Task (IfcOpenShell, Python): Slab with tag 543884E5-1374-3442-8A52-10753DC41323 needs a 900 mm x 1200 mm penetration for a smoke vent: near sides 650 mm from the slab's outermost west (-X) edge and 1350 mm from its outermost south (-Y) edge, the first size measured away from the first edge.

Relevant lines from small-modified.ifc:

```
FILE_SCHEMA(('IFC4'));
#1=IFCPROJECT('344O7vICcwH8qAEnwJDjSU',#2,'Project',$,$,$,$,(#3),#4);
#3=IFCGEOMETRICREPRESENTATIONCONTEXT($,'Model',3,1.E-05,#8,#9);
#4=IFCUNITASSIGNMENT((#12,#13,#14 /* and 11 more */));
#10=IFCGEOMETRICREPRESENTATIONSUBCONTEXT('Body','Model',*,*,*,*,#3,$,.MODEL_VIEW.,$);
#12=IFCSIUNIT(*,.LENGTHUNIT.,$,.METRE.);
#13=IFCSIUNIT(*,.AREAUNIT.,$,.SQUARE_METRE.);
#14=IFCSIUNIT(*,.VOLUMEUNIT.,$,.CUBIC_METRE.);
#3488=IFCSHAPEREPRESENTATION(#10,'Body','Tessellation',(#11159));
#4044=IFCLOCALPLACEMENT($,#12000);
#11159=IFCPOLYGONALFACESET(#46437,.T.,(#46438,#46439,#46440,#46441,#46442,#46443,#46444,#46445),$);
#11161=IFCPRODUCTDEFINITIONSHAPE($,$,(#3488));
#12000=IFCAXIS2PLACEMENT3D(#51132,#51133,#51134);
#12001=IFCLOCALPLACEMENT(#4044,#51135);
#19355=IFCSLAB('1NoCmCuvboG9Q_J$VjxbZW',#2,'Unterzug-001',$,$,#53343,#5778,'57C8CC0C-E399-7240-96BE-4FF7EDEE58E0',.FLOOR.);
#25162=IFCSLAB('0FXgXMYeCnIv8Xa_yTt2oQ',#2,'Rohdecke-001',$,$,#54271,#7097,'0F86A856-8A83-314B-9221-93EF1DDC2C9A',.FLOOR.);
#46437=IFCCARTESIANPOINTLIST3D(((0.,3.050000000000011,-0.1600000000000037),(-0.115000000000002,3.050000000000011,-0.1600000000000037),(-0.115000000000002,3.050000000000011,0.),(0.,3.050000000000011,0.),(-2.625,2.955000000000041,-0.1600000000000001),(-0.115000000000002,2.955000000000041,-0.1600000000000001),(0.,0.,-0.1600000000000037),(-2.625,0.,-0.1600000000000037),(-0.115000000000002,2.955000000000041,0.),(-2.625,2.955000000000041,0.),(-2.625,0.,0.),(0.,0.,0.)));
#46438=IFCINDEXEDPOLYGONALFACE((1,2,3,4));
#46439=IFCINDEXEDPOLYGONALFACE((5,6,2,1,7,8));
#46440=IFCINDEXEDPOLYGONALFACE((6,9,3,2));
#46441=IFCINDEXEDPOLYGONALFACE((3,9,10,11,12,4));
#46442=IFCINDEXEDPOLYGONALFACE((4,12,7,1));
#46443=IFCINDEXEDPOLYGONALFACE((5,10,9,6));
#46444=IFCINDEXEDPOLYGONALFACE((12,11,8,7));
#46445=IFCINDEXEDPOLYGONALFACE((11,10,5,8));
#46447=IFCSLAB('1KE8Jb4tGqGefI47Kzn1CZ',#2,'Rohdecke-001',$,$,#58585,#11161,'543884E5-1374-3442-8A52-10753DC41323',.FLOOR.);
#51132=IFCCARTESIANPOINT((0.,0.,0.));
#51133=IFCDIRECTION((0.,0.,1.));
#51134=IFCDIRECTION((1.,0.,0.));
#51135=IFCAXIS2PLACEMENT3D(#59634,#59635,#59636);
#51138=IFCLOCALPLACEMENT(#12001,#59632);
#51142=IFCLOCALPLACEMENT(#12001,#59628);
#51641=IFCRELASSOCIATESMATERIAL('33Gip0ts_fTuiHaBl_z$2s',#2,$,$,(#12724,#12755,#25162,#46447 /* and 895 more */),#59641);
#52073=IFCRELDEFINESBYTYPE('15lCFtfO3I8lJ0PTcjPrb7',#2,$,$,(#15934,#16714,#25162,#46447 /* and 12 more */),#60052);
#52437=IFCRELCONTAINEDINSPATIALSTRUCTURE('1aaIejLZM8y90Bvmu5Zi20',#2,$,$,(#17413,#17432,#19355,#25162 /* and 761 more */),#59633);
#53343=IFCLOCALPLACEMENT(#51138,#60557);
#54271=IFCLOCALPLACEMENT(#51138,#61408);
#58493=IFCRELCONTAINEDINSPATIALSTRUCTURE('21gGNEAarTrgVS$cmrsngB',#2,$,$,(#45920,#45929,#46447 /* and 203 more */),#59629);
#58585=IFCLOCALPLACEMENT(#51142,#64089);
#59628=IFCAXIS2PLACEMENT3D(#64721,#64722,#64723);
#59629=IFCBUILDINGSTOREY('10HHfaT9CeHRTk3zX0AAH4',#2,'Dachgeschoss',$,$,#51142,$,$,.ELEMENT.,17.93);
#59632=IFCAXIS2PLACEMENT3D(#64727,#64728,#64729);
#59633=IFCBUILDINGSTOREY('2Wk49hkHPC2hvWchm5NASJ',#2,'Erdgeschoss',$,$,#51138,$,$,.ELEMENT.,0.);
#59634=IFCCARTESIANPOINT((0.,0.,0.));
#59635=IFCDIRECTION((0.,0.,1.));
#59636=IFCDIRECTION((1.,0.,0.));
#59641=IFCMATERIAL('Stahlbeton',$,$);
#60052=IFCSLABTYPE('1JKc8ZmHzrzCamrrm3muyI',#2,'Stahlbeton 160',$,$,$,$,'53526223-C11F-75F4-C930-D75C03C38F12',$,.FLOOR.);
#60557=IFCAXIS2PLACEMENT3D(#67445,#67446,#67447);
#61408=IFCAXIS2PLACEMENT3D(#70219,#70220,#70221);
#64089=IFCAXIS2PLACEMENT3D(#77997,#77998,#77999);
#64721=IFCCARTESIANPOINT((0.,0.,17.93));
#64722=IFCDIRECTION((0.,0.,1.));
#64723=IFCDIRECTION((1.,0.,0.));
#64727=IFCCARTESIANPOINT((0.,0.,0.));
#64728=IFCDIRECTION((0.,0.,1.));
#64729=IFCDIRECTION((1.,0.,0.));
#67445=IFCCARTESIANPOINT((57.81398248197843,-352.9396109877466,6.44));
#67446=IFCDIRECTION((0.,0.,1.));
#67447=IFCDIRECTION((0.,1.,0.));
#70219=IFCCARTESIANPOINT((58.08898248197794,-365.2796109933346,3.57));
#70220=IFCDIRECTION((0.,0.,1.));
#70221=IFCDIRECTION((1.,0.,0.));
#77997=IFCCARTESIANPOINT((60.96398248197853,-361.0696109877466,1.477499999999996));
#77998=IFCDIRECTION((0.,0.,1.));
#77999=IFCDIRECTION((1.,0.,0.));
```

```python
import numpy as np
import ifcopenshell
import ifcopenshell.api.feature
import ifcopenshell.api.geometry
import ifcopenshell.api.root
import ifcopenshell.geom
import ifcopenshell.util.placement
import ifcopenshell.util.representation
import ifcopenshell.util.shape
import ifcopenshell.util.unit

model = ifcopenshell.open("small-modified.ifc")
unit_scale = ifcopenshell.util.unit.calculate_unit_scale(model)
settings = ifcopenshell.geom.settings()


def volume(element):
    """Net volume in cubic metres, openings subtracted."""
    shape = ifcopenshell.geom.create_shape(settings, element)
    return ifcopenshell.util.shape.get_volume(shape.geometry)


slab = model.by_id(46447)
before = volume(slab)

# Extent in the slab's own axes, in metres. The edges named are its -X and -Y sides.
slab_shape = ifcopenshell.geom.create_shape(settings, slab)
vertices = ifcopenshell.util.shape.get_vertices(slab_shape.geometry)
x_min, y_min, bottom = vertices.min(axis=0)
top = vertices[:, 2].max()

opening = ifcopenshell.api.root.create_entity(model, ifc_class="IfcOpeningElement", name="Smoke vent opening", predefined_type="OPENING")
context = ifcopenshell.util.representation.get_context(model, "Model", "Body", "MODEL_VIEW")
width, depth = 0.9, 1.2
outline = [(0.0, 0.0), (width, 0.0), (width, depth), (0.0, depth), (0.0, 0.0)]
# Overshoot both faces by 50 mm so the cut is clean.
shape = ifcopenshell.api.geometry.add_slab_representation(
    model, context=context, depth=top - bottom + 0.1, polyline=outline
)
ifcopenshell.api.geometry.assign_representation(model, product=opening, representation=shape)

matrix = ifcopenshell.util.placement.get_local_placement(slab.ObjectPlacement)
matrix[:, 3] = matrix @ np.append(np.array([x_min + 0.65, y_min + 1.35, bottom - 0.05]) / unit_scale, 1.0)
ifcopenshell.api.geometry.edit_object_placement(model, product=opening, matrix=matrix, is_si=False)
ifcopenshell.api.feature.add_feature(model, feature=opening, element=slab)

after = volume(slab)

print(f"slab volume {before:.3f} -> {after:.3f} m3")

model.write("small-modified-out.ifc")
```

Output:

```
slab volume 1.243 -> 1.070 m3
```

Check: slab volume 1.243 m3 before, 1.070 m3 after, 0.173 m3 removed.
